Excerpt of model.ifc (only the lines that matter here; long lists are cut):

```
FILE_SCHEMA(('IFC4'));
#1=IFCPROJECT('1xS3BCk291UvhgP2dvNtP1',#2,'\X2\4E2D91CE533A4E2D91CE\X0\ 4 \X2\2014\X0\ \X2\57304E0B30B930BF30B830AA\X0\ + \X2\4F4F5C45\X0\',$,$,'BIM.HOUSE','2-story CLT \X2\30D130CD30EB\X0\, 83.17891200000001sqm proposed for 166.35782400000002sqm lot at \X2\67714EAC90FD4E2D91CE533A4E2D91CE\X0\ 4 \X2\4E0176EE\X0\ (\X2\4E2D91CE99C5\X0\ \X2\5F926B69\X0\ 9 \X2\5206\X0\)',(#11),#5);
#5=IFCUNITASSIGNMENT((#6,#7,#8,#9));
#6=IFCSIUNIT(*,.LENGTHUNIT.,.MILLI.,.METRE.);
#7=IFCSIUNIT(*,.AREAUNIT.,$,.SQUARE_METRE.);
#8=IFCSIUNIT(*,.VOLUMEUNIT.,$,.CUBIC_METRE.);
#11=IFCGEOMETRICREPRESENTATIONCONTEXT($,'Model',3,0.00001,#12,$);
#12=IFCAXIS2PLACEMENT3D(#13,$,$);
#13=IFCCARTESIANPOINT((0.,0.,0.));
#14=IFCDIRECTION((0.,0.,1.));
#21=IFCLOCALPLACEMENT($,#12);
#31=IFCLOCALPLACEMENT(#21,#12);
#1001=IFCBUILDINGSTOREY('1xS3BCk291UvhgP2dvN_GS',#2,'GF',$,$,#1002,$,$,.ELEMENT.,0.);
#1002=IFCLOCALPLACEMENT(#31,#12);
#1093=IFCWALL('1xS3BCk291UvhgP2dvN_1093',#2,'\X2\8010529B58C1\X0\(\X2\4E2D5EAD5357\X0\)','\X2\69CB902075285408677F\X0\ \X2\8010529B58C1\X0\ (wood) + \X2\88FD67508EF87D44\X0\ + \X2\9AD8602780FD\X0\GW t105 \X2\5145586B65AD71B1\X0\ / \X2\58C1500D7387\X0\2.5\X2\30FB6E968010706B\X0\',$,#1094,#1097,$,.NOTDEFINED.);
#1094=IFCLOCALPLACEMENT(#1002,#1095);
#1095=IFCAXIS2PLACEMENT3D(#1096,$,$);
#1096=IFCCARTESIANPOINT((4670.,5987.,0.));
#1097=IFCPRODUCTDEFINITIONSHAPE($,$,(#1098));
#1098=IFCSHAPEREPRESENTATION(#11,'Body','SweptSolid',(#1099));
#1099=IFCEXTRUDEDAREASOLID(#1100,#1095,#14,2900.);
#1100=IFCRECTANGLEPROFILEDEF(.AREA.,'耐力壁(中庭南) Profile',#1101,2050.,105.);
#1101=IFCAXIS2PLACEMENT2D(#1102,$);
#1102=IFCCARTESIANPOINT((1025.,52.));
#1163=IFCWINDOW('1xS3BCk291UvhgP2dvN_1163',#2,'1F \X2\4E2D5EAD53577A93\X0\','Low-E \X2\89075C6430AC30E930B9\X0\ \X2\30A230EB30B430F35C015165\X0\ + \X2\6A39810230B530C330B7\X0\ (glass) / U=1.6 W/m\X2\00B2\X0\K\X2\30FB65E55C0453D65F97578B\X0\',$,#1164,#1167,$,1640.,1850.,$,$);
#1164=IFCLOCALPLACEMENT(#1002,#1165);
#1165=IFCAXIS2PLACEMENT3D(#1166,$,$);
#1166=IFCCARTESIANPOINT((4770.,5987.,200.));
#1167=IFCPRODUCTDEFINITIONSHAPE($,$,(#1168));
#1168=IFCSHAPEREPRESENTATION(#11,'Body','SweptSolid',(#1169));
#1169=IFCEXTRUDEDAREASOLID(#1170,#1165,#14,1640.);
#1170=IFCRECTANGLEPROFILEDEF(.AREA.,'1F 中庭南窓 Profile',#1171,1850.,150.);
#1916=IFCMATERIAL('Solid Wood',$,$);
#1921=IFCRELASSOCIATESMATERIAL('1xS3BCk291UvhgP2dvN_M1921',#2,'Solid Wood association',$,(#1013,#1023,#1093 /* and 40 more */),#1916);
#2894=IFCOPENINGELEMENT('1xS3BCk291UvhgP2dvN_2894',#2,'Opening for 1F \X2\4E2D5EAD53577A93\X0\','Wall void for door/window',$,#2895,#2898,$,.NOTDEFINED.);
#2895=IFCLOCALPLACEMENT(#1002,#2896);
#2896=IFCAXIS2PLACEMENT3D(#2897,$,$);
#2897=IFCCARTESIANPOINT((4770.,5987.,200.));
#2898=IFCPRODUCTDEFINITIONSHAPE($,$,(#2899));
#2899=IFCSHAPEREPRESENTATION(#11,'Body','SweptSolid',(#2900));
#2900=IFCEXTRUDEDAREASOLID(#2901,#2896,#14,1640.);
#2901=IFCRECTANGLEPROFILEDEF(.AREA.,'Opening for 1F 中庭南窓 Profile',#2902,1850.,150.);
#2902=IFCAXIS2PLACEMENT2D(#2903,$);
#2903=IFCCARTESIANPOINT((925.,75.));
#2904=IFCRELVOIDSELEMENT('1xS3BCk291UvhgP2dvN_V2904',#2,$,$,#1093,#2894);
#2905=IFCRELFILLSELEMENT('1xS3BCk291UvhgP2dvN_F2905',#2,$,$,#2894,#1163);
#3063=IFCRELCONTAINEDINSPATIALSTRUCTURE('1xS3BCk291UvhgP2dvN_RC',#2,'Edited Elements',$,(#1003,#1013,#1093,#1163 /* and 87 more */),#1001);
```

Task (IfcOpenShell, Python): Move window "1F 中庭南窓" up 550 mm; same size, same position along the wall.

```python
import numpy as np
import ifcopenshell
import ifcopenshell.api.geometry
import ifcopenshell.util.placement
import ifcopenshell.util.unit

model = ifcopenshell.open("model.ifc")
unit_scale = ifcopenshell.util.unit.calculate_unit_scale(model)

window = model.by_id(1163)
opening = window.FillsVoids[0].RelatingOpeningElement
dz = 0.55 / unit_scale

shift = np.array([0.0, 0.0, dz])
# The window is not placed relative to its opening, so move both.
for product in (opening, window):
    matrix = ifcopenshell.util.placement.get_local_placement(product.ObjectPlacement)
    matrix[:3, 3] += shift
    ifcopenshell.api.geometry.edit_object_placement(model, product=product, matrix=matrix, is_si=False)

print(f"moved by {dz * unit_scale:+.3f} m")

model.write("model_updated.ifc")
```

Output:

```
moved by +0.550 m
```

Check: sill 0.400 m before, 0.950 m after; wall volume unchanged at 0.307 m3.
